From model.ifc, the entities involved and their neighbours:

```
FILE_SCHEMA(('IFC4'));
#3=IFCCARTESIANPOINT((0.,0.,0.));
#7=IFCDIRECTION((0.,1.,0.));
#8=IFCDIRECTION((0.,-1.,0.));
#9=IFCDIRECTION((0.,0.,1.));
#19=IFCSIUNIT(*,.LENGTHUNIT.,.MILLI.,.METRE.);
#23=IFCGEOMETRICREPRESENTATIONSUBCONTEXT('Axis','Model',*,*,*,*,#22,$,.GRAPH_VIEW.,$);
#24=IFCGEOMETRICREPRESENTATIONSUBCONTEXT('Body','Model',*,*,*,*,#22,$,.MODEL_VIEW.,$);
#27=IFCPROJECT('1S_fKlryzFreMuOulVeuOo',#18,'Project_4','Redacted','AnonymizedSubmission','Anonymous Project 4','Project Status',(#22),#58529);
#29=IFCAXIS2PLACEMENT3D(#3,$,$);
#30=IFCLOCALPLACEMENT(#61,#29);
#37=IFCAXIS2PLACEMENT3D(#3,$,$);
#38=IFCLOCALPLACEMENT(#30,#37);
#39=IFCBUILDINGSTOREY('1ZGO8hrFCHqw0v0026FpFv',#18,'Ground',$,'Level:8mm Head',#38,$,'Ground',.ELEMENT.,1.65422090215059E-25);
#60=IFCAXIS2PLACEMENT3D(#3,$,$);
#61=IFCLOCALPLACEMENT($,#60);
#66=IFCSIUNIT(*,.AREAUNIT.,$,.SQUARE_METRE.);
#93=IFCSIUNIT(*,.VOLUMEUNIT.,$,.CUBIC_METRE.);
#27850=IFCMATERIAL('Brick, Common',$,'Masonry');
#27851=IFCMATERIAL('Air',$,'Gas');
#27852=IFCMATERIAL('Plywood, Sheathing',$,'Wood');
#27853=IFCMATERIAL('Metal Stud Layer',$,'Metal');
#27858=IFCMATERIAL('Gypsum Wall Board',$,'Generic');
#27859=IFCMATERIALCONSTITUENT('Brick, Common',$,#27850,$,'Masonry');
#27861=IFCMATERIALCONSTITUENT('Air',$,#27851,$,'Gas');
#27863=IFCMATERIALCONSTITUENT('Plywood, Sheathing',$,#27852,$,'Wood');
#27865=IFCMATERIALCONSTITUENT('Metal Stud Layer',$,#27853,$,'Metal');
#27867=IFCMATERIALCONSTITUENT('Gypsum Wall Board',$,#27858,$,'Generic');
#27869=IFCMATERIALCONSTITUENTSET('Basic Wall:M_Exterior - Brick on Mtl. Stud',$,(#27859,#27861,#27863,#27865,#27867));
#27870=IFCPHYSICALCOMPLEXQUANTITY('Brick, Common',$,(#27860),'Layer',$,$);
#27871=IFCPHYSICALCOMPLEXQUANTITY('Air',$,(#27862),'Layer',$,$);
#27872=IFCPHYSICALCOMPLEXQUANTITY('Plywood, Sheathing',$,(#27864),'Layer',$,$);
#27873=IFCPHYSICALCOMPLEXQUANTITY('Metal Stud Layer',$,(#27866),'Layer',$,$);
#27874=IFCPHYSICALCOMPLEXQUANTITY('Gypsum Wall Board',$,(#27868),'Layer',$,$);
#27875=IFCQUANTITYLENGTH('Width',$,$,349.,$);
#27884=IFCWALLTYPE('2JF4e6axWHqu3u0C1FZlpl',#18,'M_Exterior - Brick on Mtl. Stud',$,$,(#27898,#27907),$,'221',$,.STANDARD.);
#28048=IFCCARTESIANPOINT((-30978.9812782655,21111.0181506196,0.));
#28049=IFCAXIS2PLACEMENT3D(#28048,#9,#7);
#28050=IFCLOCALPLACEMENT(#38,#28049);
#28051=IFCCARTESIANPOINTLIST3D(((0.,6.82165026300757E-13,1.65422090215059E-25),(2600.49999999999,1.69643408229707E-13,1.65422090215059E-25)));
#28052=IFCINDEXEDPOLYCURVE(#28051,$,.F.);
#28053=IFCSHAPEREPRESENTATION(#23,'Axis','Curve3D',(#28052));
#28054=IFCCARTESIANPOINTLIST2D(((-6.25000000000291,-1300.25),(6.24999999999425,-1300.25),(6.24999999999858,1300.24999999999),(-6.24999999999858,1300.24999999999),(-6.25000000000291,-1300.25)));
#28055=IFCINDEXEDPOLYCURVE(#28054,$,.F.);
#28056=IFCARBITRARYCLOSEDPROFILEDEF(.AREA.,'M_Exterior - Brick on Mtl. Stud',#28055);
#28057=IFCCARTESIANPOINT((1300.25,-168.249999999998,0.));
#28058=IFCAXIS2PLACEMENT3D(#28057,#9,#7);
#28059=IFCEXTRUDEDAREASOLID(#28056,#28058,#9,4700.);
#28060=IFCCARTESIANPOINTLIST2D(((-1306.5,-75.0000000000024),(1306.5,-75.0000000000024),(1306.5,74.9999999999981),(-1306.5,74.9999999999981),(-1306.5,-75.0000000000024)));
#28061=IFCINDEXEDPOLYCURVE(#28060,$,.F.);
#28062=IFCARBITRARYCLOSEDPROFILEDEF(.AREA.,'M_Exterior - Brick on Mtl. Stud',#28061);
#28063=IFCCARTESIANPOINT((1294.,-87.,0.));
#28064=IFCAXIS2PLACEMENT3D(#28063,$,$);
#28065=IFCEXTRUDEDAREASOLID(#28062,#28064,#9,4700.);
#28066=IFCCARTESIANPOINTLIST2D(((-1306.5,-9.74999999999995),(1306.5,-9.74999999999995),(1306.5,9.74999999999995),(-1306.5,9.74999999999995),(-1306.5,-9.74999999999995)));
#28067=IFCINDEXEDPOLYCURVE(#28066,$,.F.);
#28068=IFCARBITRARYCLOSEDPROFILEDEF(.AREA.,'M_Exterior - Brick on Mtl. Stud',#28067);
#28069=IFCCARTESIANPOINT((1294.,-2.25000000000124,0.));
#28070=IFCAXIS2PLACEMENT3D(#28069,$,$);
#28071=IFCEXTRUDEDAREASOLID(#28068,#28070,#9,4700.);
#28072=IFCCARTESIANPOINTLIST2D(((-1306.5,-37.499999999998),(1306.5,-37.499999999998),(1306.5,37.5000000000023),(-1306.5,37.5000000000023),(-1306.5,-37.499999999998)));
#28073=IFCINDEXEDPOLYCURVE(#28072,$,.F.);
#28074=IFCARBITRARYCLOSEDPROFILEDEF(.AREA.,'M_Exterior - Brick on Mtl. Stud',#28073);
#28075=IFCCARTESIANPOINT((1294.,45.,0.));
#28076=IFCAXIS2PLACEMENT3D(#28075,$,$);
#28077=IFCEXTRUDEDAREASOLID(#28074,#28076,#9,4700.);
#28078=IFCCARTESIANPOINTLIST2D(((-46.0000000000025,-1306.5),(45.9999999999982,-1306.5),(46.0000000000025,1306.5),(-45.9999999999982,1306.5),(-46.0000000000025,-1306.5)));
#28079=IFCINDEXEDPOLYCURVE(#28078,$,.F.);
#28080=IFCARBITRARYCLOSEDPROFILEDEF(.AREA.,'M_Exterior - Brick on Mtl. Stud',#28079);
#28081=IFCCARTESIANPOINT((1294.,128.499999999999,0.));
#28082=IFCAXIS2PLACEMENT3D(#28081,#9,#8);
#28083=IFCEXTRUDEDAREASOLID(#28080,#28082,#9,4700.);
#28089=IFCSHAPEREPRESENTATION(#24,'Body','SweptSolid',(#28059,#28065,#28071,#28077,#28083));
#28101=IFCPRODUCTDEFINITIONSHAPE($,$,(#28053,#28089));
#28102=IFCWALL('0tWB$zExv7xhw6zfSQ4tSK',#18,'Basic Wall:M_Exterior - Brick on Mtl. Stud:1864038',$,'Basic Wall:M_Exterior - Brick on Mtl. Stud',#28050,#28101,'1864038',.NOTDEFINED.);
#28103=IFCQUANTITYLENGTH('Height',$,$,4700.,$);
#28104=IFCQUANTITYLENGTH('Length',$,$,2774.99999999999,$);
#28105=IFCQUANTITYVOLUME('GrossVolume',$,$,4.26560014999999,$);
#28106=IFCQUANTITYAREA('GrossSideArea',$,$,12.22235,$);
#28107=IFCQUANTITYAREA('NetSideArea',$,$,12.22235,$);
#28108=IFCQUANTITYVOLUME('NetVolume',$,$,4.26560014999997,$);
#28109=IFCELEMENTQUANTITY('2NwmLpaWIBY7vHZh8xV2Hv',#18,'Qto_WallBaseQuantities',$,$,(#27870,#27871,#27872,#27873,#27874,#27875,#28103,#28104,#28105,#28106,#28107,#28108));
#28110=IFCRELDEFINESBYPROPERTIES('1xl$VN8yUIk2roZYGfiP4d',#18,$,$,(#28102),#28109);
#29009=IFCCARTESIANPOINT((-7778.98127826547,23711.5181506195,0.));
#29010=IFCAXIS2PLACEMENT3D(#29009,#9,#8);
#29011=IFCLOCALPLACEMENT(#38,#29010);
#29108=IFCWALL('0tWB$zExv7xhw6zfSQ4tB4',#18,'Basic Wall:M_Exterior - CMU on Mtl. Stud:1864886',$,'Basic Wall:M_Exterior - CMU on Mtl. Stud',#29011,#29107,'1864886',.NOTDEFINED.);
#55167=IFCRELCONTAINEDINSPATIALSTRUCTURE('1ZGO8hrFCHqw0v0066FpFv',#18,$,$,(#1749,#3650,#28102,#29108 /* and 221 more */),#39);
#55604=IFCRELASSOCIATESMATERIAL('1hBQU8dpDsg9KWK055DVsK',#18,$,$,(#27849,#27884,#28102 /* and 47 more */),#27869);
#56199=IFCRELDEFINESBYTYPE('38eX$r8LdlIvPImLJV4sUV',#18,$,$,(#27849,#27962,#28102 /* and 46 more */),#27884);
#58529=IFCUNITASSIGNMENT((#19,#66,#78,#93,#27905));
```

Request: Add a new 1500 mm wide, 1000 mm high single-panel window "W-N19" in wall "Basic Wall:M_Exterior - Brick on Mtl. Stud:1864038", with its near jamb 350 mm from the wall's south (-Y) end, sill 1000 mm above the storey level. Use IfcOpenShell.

```python
import numpy as np
import ifcopenshell
import ifcopenshell.api.feature
import ifcopenshell.api.geometry
import ifcopenshell.api.pset
import ifcopenshell.api.root
import ifcopenshell.api.spatial
import ifcopenshell.geom
import ifcopenshell.util.element
import ifcopenshell.util.placement
import ifcopenshell.util.representation
import ifcopenshell.util.shape
import ifcopenshell.util.unit

model = ifcopenshell.open("model.ifc")
unit_scale = ifcopenshell.util.unit.calculate_unit_scale(model)
area_scale = ifcopenshell.util.unit.calculate_unit_scale(model, "AREAUNIT")
volume_scale = ifcopenshell.util.unit.calculate_unit_scale(model, "VOLUMEUNIT")
settings = ifcopenshell.geom.settings()


def volume(element):
    """Net volume in cubic metres, openings subtracted."""
    shape = ifcopenshell.geom.create_shape(settings, element)
    return ifcopenshell.util.shape.get_volume(shape.geometry)


wall = model.by_guid("0tWB$zExv7xhw6zfSQ4tSK")
storey = ifcopenshell.util.element.get_container(wall, ifc_class="IfcBuildingStorey")
context = ifcopenshell.util.representation.get_context(model, "Model", "Body", "MODEL_VIEW")
before = volume(wall)

width, height, from_end, sill = 1.5, 1, 0.35, 1  # metres

# The wall runs along its own X axis, and the end named is its -X end.
wall_shape = ifcopenshell.geom.create_shape(settings, wall)
x, y, z = ifcopenshell.util.shape.get_vertices(wall_shape.geometry).T
start = x.min() + from_end
face, thickness = float(y.min()), float(y.max() - y.min())
wall_matrix = ifcopenshell.util.placement.get_local_placement(wall.ObjectPlacement)
level = ifcopenshell.util.placement.get_local_placement(storey.ObjectPlacement)[2, 3]


def in_wall(x, y):
    """Placement at x, y metres in the wall's axes, at sill height."""
    matrix = wall_matrix.copy()
    matrix[:, 3] = wall_matrix @ np.array([x / unit_scale, y / unit_scale, 0.0, 1.0])
    matrix[2, 3] = level + sill / unit_scale
    return matrix


# Opening: a box that overshoots both wall faces by 50 mm.
opening = ifcopenshell.api.root.create_entity(model, ifc_class="IfcOpeningElement", predefined_type="OPENING")
box = ifcopenshell.api.geometry.add_wall_representation(
    model, context=context, length=width, height=height, thickness=thickness + 0.1
)
ifcopenshell.api.geometry.assign_representation(model, product=opening, representation=box)
ifcopenshell.api.geometry.edit_object_placement(model, product=opening, matrix=in_wall(start, face - 0.05), is_si=False)
ifcopenshell.api.feature.add_feature(model, feature=opening, element=wall)

window = ifcopenshell.api.root.create_entity(model, ifc_class="IfcWindow", name="W-N19", predefined_type="WINDOW")
window.OverallWidth, window.OverallHeight = width / unit_scale, height / unit_scale
window.PartitioningType = "SINGLE_PANEL"
body = ifcopenshell.api.geometry.add_window_representation(
    model,
    context=context,
    overall_width=window.OverallWidth,
    overall_height=window.OverallHeight,
    partition_type="SINGLE_PANEL",
)
ifcopenshell.api.geometry.assign_representation(model, product=window, representation=body)
ifcopenshell.api.spatial.assign_container(model, products=[window], relating_structure=storey)
ifcopenshell.api.feature.add_filling(model, opening=opening, element=window)

# Centre the window in the wall's thickness.
ifcopenshell.api.geometry.edit_object_placement(model, product=window, matrix=in_wall(start, face), is_si=False)
window_shape = ifcopenshell.geom.create_shape(settings, window)
depth = ifcopenshell.util.shape.get_vertices(window_shape.geometry)[:, 1]
offset = face + thickness / 2 - (depth.min() + depth.max()) / 2
ifcopenshell.api.geometry.edit_object_placement(model, product=window, matrix=in_wall(start, offset), is_si=False)

after = volume(wall)

# Update the wall's stored quantities.
qto = model.by_id(ifcopenshell.util.element.get_pset(wall, "Qto_WallBaseQuantities", should_inherit=False)["id"])
ifcopenshell.api.pset.edit_qto(model, qto=qto, properties={
    "NetSideArea": after / thickness / area_scale,
    "NetVolume": after / volume_scale,
})

print(f"wall volume {before:.3f} -> {after:.3f} m3")

model.write("model_edited.ifc")
```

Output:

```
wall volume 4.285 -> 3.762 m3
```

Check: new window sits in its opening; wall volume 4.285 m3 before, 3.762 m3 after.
